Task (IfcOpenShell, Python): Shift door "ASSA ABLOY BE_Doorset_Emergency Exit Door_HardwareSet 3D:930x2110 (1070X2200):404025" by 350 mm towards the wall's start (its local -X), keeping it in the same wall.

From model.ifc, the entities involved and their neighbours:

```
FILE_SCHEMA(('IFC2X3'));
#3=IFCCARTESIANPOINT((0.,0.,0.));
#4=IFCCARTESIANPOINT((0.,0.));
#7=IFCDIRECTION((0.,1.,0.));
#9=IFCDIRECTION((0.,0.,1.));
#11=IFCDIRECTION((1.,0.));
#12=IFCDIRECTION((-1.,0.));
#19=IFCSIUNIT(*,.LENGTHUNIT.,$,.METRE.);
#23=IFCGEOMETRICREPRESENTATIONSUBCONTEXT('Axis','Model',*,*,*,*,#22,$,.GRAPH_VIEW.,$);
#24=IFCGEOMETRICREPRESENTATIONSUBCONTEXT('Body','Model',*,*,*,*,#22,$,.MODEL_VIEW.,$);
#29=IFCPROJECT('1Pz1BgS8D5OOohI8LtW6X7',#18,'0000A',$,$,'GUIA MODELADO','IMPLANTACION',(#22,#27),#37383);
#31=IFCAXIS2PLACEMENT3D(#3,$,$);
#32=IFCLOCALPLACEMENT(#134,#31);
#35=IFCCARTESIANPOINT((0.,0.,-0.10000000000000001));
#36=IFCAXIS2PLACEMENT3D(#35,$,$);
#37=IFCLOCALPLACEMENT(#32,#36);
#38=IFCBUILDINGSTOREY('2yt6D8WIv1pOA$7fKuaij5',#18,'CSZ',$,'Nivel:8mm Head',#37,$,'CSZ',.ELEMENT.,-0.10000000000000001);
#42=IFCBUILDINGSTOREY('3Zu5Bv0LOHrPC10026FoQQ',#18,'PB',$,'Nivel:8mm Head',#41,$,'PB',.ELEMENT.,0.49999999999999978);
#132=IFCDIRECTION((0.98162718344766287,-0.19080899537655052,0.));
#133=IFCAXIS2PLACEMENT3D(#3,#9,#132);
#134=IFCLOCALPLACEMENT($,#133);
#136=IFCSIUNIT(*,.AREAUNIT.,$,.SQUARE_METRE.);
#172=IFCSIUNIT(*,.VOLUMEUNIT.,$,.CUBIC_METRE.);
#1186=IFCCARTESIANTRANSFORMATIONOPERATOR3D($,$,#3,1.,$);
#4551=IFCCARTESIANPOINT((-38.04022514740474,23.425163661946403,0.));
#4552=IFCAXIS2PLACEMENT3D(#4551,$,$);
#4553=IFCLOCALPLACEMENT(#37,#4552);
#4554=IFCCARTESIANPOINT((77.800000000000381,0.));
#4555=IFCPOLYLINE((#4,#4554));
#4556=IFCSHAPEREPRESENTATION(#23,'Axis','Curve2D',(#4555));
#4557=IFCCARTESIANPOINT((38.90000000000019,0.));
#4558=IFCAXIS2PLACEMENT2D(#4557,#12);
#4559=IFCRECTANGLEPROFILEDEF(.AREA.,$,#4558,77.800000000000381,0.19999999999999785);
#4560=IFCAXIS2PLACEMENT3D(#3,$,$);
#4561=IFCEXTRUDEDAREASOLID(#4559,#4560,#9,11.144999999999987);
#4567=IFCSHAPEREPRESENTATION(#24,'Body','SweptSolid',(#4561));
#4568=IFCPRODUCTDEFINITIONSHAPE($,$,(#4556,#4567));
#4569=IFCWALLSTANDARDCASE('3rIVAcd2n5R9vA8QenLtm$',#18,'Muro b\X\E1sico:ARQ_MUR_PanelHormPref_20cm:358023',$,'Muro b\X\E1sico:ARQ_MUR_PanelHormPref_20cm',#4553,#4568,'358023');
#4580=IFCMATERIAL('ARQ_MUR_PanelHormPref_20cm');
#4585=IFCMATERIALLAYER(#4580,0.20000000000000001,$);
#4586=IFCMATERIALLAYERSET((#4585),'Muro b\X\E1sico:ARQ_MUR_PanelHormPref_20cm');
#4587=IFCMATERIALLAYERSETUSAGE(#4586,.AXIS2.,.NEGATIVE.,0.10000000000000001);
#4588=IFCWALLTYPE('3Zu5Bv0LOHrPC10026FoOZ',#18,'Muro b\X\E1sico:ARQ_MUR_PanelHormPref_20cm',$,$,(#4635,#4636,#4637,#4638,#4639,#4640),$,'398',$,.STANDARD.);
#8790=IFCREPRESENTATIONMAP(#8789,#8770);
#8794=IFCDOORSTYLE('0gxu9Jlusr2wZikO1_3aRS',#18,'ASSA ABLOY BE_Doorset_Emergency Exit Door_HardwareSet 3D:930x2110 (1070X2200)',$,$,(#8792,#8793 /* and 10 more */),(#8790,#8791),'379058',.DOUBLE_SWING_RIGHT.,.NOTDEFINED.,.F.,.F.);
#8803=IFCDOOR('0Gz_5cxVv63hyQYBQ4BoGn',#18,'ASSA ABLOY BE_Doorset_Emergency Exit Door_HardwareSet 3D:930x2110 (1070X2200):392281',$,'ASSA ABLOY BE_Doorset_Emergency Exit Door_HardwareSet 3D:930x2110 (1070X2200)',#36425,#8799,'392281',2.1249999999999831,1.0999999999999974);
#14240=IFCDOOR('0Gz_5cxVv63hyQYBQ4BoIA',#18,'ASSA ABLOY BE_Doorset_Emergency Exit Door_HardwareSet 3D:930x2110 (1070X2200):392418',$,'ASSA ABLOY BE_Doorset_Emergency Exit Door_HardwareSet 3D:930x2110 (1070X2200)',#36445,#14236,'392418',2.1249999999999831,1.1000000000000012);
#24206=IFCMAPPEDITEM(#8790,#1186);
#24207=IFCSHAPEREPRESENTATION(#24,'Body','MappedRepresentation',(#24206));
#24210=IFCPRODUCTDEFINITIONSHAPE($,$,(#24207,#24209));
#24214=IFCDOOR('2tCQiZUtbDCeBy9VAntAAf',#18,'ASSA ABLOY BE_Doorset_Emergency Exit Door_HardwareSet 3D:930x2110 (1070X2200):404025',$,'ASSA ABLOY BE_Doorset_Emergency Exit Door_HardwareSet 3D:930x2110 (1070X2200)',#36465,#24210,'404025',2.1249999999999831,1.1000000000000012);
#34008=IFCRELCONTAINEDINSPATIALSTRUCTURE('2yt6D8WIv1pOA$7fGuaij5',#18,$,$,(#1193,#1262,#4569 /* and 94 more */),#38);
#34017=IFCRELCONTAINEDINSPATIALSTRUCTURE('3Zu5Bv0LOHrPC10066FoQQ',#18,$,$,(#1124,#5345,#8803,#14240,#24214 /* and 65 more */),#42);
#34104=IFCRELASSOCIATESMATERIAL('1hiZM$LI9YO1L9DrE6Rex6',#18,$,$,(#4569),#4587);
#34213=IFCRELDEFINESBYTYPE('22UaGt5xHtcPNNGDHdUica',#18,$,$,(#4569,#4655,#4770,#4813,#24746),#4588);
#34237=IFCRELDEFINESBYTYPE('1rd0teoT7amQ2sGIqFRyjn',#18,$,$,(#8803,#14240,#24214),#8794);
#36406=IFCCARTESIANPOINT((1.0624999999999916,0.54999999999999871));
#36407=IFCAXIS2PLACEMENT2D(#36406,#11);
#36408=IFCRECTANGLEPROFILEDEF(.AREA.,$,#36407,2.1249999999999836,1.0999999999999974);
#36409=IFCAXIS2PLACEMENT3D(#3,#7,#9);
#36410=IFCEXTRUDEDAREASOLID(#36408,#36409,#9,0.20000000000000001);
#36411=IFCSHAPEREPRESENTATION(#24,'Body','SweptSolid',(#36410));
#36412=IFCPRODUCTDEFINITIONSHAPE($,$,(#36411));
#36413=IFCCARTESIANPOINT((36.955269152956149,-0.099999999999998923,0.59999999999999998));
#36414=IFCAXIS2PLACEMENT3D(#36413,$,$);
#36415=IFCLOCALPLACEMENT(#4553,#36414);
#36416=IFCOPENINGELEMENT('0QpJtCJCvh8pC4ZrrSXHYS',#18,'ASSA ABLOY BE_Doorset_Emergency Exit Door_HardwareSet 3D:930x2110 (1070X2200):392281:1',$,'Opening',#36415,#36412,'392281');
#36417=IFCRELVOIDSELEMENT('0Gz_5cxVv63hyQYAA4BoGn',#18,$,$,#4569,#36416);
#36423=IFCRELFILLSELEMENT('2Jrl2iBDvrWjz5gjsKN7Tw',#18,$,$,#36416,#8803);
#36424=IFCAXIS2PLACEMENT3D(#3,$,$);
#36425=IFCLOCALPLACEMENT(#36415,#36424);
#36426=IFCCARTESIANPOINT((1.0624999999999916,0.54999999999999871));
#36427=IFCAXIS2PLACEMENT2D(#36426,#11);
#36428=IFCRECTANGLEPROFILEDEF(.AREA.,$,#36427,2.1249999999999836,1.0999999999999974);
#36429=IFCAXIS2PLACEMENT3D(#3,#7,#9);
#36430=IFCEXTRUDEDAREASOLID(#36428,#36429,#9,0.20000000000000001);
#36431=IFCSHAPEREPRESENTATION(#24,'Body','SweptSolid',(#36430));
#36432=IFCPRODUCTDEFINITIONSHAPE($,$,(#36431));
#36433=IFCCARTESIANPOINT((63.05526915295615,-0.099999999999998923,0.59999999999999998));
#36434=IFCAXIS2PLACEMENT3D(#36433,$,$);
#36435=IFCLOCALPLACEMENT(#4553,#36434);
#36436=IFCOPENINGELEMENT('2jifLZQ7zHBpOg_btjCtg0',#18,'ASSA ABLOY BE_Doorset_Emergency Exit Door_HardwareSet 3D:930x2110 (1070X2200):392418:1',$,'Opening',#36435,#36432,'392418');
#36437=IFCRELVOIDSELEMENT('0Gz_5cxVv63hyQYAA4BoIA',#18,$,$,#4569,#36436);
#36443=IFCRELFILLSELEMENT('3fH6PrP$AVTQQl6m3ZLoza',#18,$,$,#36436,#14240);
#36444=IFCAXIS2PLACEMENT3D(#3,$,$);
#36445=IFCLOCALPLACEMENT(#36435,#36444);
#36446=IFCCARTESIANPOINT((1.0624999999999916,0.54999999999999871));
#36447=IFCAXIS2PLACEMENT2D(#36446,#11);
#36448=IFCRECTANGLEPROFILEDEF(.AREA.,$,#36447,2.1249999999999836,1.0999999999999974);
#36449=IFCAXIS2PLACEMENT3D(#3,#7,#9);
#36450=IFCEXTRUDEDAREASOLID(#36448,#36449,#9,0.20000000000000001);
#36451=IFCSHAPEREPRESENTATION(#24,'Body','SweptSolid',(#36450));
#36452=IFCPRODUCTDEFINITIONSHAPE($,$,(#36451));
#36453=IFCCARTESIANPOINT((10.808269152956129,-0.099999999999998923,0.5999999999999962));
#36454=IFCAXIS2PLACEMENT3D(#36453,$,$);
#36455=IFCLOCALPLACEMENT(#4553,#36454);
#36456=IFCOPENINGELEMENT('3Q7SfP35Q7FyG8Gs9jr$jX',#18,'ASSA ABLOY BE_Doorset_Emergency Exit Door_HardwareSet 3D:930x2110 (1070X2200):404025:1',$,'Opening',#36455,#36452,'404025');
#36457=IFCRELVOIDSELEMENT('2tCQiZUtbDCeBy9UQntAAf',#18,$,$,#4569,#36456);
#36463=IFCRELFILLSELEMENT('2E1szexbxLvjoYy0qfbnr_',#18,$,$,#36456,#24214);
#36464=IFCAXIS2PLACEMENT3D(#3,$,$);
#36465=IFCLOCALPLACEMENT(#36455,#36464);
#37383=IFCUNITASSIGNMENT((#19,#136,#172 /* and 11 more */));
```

```python
import ifcopenshell
import ifcopenshell.api.geometry
import ifcopenshell.util.placement
import ifcopenshell.util.unit

model = ifcopenshell.open("model.ifc")
unit_scale = ifcopenshell.util.unit.calculate_unit_scale(model)

door = model.by_guid("2tCQiZUtbDCeBy9VAntAAf")
opening = door.FillsVoids[0].RelatingOpeningElement
wall = opening.VoidsElements[0].RelatingBuildingElement

wall_matrix = ifcopenshell.util.placement.get_local_placement(wall.ObjectPlacement)
shift = wall_matrix[:3, 0] * -0.35 / unit_scale
before = ifcopenshell.util.placement.get_local_placement(door.ObjectPlacement)[:3, 3].copy()

# The door is placed relative to its opening, so it follows when the opening moves.
matrix = ifcopenshell.util.placement.get_local_placement(opening.ObjectPlacement)
matrix[:3, 3] += shift
ifcopenshell.api.geometry.edit_object_placement(
    model, product=opening, matrix=matrix, is_si=False, should_transform_children=True
)

after = ifcopenshell.util.placement.get_local_placement(door.ObjectPlacement)[:3, 3]
print("door moved by", (after - before).round(3) + 0.0)

model.write("model-out.ifc")
```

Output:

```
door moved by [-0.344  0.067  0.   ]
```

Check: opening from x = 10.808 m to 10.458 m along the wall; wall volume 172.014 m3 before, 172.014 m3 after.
